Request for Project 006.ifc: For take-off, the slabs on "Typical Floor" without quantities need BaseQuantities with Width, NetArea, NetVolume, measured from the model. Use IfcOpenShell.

First a look at what the model holds.

```python
import ifcopenshell
import ifcopenshell.util.element
import ifcopenshell.util.unit

model = ifcopenshell.open("Project 006.ifc")
print(model.schema)
for unit_type in ("LENGTHUNIT", "AREAUNIT", "VOLUMEUNIT"):
    print(unit_type, ifcopenshell.util.unit.calculate_unit_scale(model, unit_type))
storey = next(s for s in model.by_type("IfcBuildingStorey") if s.Name == "Typical Floor")
slabs = [e for e in ifcopenshell.util.element.get_decomposition(storey) if e.is_a("IfcSlab")]
for e in sorted(slabs, key=lambda e: e.id()):
    print(e.id(), e.is_a(), e.Name, list(ifcopenshell.util.element.get_psets(e, qtos_only=True)), sep=" | ")
```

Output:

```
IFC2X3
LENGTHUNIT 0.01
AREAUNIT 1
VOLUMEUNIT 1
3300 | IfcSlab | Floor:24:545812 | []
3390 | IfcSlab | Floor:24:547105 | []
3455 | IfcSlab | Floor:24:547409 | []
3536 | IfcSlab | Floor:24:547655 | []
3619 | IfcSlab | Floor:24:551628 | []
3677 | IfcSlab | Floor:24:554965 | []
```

```python
import ifcopenshell
import ifcopenshell.api.pset
import ifcopenshell.geom
import ifcopenshell.util.element
import ifcopenshell.util.shape
import ifcopenshell.util.unit

model = ifcopenshell.open("Project 006.ifc")
unit_scale = ifcopenshell.util.unit.calculate_unit_scale(model)
area_scale = ifcopenshell.util.unit.calculate_unit_scale(model, "AREAUNIT")
volume_scale = ifcopenshell.util.unit.calculate_unit_scale(model, "VOLUMEUNIT")
settings = ifcopenshell.geom.settings()

storey = next(s for s in model.by_type("IfcBuildingStorey") if s.Name == "Typical Floor")
slabs = [e for e in ifcopenshell.util.element.get_decomposition(storey) if e.is_a("IfcSlab")]

for e in sorted(slabs, key=lambda e: e.id()):
    if ifcopenshell.util.element.get_psets(e, qtos_only=True, should_inherit=False):
        continue
    # Geometry comes back in metres, in the element's own axes.
    shape = ifcopenshell.geom.create_shape(settings, e)
    values = {
        "Width": ifcopenshell.util.shape.get_z(shape.geometry) / unit_scale,
        "NetArea": ifcopenshell.util.shape.get_footprint_area(shape.geometry) / area_scale,
        "NetVolume": ifcopenshell.util.shape.get_volume(shape.geometry) / volume_scale,
    }
    qto = ifcopenshell.api.pset.add_qto(model, product=e, name="BaseQuantities")
    ifcopenshell.api.pset.edit_qto(model, qto=qto, properties=values)
    print(e.id(), {k: round(v, 3) for k, v in values.items()})

model.write("Project 006-out.ifc")
```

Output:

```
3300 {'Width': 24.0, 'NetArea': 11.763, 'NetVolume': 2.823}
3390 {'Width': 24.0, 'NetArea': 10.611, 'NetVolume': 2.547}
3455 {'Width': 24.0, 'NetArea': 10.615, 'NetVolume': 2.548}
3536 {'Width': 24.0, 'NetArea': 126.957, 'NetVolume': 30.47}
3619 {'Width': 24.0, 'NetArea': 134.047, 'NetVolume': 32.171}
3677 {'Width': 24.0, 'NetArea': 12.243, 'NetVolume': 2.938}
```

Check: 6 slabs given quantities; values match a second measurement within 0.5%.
